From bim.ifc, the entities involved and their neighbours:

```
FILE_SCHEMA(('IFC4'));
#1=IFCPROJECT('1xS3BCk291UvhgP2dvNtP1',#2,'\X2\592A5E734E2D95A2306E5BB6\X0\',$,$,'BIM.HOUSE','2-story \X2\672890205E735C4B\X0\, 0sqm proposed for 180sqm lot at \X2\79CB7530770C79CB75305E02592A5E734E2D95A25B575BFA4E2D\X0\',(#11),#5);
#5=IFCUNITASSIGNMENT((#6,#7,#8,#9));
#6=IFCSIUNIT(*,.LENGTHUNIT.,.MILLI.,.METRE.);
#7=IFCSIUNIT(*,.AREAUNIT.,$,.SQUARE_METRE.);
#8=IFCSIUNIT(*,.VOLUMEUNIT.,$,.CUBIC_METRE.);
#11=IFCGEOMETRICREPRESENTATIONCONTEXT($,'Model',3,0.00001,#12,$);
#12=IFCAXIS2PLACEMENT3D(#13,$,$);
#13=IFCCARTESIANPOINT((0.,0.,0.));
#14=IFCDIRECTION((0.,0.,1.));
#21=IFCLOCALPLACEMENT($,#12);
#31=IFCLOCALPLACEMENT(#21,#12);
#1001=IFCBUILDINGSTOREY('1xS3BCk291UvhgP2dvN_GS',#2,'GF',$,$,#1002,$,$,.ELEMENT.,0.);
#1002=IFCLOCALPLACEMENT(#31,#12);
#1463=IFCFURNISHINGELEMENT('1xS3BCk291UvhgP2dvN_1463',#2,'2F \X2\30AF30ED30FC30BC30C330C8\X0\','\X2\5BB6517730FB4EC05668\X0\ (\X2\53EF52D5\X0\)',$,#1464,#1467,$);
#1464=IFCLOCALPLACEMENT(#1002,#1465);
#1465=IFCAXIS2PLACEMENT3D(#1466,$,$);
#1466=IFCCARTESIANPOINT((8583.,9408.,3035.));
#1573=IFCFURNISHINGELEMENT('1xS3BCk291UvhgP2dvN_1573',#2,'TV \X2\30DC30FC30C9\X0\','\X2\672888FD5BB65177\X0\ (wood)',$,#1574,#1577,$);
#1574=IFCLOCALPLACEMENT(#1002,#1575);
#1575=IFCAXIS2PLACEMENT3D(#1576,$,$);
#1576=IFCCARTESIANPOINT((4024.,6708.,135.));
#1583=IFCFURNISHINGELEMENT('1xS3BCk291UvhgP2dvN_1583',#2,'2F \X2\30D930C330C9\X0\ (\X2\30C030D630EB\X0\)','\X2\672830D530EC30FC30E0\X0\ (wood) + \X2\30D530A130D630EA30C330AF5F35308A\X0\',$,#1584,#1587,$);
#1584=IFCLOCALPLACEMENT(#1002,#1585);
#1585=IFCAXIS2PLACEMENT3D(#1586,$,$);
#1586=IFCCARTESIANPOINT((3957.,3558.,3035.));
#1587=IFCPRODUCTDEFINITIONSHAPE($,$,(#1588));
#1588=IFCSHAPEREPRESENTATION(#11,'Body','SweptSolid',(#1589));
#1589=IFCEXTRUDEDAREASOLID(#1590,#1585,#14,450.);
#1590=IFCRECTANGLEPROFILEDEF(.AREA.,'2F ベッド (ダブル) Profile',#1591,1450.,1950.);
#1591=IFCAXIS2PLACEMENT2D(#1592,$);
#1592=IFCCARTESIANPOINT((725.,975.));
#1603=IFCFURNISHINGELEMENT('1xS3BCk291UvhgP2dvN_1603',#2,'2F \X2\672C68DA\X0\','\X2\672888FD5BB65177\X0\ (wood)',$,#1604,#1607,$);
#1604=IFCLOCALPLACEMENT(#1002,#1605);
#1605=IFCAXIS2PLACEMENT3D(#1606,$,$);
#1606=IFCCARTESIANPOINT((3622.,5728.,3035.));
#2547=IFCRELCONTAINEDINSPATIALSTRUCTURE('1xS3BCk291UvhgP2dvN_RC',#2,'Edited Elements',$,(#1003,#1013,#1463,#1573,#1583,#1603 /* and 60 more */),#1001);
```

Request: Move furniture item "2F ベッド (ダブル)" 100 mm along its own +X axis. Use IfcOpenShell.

```python
import ifcopenshell
import ifcopenshell.api.geometry
import ifcopenshell.util.placement

model = ifcopenshell.open("bim.ifc")

item = model.by_guid("1xS3BCk291UvhgP2dvN_1583")
matrix = ifcopenshell.util.placement.get_local_placement(item.ObjectPlacement)
matrix[:3, 3] += matrix[:3, 0] * 100.0
ifcopenshell.api.geometry.edit_object_placement(model, product=item, matrix=matrix, is_si=False)

print(ifcopenshell.util.placement.get_local_placement(item.ObjectPlacement).round(3) + 0.0)

model.write("bim_rev.ifc")
```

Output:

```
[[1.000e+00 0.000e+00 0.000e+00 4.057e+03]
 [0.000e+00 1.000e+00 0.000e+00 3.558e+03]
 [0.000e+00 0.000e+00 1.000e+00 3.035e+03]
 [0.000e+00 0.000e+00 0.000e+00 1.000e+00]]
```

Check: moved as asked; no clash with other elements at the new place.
